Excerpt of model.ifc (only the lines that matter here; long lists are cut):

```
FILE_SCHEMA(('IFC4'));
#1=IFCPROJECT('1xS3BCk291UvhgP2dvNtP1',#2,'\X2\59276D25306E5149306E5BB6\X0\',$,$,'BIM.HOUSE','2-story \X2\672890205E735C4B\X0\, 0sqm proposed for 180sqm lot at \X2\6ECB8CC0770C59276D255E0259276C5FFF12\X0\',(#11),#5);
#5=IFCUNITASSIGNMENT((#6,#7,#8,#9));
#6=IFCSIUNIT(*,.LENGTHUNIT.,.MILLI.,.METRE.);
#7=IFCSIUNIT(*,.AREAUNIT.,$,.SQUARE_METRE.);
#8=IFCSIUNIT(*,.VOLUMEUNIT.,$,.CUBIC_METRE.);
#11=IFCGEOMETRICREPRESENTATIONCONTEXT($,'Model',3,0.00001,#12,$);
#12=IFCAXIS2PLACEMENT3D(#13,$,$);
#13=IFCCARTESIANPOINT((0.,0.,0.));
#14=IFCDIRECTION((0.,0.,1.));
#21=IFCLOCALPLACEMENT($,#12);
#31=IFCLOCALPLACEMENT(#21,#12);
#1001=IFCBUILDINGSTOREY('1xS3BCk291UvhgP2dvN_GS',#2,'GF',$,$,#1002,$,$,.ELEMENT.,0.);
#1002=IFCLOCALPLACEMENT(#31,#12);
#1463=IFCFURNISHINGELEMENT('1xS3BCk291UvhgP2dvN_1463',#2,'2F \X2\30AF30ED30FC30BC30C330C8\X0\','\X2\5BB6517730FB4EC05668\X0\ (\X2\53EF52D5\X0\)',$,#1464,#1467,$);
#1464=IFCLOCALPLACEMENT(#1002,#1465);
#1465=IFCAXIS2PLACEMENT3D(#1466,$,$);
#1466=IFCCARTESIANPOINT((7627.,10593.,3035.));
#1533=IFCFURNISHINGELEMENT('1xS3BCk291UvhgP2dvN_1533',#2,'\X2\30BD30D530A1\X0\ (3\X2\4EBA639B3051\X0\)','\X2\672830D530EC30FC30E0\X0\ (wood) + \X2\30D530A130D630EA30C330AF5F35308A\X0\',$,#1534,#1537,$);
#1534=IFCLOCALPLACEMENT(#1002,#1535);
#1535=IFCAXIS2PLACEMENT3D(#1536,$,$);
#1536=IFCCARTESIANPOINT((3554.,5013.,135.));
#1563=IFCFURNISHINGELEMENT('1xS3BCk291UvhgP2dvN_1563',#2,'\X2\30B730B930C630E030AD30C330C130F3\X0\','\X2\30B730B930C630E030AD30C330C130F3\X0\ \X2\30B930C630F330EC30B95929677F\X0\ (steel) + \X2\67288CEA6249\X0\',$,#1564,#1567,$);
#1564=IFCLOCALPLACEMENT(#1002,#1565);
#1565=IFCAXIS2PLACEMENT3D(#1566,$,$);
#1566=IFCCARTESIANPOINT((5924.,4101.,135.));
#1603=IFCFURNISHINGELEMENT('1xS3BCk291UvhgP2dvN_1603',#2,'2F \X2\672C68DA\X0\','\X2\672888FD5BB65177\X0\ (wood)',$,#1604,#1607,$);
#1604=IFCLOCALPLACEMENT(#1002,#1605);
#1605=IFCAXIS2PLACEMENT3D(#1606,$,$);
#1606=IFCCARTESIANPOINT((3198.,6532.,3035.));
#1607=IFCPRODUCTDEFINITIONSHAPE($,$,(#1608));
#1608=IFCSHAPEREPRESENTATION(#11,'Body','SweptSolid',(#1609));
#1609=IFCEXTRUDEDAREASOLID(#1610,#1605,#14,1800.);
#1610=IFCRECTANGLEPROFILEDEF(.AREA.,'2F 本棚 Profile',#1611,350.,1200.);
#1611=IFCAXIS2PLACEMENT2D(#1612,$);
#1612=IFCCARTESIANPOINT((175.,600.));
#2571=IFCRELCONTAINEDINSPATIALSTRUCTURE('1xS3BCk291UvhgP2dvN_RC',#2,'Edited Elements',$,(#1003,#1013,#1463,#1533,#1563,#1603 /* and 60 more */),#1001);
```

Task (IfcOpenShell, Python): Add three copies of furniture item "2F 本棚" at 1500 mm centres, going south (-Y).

```python
import numpy as np
import ifcopenshell
import ifcopenshell.api.geometry
import ifcopenshell.api.root
import ifcopenshell.util.element
import ifcopenshell.util.placement

model = ifcopenshell.open("model.ifc")


def reuse_history(source, copy):
    """copy_class also copies each property set's owner history, people and application; keep the originals."""
    for rel in copy.IsDefinedBy:
        if rel.is_a("IfcRelDefinesByProperties") and (history := rel.RelatingPropertyDefinition.OwnerHistory):
            rel.RelatingPropertyDefinition.OwnerHistory = source.OwnerHistory
            ifcopenshell.util.element.remove_deep2(model, history)


source = model.by_guid("1xS3BCk291UvhgP2dvN_1603")
base = ifcopenshell.util.placement.get_local_placement(source.ObjectPlacement)
step = np.array([0.0, -1.0, 0.0]) * 1500.0

for i in range(1, 4):
    copy = ifcopenshell.api.root.copy_class(model, product=source)
    copy.Representation = ifcopenshell.util.element.copy_deep(
        model, source.Representation, exclude=["IfcGeometricRepresentationContext", "IfcRepresentationMap"]
    )
    reuse_history(source, copy)
    matrix = base.copy()
    matrix[:3, 3] += i * step
    print("added at", matrix[:3, 3].round(3) + 0.0)
    ifcopenshell.api.geometry.edit_object_placement(model, product=copy, matrix=matrix, is_si=False)

model.write("model_edited.ifc")
```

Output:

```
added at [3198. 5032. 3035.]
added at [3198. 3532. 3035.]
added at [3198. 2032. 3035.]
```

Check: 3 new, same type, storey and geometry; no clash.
